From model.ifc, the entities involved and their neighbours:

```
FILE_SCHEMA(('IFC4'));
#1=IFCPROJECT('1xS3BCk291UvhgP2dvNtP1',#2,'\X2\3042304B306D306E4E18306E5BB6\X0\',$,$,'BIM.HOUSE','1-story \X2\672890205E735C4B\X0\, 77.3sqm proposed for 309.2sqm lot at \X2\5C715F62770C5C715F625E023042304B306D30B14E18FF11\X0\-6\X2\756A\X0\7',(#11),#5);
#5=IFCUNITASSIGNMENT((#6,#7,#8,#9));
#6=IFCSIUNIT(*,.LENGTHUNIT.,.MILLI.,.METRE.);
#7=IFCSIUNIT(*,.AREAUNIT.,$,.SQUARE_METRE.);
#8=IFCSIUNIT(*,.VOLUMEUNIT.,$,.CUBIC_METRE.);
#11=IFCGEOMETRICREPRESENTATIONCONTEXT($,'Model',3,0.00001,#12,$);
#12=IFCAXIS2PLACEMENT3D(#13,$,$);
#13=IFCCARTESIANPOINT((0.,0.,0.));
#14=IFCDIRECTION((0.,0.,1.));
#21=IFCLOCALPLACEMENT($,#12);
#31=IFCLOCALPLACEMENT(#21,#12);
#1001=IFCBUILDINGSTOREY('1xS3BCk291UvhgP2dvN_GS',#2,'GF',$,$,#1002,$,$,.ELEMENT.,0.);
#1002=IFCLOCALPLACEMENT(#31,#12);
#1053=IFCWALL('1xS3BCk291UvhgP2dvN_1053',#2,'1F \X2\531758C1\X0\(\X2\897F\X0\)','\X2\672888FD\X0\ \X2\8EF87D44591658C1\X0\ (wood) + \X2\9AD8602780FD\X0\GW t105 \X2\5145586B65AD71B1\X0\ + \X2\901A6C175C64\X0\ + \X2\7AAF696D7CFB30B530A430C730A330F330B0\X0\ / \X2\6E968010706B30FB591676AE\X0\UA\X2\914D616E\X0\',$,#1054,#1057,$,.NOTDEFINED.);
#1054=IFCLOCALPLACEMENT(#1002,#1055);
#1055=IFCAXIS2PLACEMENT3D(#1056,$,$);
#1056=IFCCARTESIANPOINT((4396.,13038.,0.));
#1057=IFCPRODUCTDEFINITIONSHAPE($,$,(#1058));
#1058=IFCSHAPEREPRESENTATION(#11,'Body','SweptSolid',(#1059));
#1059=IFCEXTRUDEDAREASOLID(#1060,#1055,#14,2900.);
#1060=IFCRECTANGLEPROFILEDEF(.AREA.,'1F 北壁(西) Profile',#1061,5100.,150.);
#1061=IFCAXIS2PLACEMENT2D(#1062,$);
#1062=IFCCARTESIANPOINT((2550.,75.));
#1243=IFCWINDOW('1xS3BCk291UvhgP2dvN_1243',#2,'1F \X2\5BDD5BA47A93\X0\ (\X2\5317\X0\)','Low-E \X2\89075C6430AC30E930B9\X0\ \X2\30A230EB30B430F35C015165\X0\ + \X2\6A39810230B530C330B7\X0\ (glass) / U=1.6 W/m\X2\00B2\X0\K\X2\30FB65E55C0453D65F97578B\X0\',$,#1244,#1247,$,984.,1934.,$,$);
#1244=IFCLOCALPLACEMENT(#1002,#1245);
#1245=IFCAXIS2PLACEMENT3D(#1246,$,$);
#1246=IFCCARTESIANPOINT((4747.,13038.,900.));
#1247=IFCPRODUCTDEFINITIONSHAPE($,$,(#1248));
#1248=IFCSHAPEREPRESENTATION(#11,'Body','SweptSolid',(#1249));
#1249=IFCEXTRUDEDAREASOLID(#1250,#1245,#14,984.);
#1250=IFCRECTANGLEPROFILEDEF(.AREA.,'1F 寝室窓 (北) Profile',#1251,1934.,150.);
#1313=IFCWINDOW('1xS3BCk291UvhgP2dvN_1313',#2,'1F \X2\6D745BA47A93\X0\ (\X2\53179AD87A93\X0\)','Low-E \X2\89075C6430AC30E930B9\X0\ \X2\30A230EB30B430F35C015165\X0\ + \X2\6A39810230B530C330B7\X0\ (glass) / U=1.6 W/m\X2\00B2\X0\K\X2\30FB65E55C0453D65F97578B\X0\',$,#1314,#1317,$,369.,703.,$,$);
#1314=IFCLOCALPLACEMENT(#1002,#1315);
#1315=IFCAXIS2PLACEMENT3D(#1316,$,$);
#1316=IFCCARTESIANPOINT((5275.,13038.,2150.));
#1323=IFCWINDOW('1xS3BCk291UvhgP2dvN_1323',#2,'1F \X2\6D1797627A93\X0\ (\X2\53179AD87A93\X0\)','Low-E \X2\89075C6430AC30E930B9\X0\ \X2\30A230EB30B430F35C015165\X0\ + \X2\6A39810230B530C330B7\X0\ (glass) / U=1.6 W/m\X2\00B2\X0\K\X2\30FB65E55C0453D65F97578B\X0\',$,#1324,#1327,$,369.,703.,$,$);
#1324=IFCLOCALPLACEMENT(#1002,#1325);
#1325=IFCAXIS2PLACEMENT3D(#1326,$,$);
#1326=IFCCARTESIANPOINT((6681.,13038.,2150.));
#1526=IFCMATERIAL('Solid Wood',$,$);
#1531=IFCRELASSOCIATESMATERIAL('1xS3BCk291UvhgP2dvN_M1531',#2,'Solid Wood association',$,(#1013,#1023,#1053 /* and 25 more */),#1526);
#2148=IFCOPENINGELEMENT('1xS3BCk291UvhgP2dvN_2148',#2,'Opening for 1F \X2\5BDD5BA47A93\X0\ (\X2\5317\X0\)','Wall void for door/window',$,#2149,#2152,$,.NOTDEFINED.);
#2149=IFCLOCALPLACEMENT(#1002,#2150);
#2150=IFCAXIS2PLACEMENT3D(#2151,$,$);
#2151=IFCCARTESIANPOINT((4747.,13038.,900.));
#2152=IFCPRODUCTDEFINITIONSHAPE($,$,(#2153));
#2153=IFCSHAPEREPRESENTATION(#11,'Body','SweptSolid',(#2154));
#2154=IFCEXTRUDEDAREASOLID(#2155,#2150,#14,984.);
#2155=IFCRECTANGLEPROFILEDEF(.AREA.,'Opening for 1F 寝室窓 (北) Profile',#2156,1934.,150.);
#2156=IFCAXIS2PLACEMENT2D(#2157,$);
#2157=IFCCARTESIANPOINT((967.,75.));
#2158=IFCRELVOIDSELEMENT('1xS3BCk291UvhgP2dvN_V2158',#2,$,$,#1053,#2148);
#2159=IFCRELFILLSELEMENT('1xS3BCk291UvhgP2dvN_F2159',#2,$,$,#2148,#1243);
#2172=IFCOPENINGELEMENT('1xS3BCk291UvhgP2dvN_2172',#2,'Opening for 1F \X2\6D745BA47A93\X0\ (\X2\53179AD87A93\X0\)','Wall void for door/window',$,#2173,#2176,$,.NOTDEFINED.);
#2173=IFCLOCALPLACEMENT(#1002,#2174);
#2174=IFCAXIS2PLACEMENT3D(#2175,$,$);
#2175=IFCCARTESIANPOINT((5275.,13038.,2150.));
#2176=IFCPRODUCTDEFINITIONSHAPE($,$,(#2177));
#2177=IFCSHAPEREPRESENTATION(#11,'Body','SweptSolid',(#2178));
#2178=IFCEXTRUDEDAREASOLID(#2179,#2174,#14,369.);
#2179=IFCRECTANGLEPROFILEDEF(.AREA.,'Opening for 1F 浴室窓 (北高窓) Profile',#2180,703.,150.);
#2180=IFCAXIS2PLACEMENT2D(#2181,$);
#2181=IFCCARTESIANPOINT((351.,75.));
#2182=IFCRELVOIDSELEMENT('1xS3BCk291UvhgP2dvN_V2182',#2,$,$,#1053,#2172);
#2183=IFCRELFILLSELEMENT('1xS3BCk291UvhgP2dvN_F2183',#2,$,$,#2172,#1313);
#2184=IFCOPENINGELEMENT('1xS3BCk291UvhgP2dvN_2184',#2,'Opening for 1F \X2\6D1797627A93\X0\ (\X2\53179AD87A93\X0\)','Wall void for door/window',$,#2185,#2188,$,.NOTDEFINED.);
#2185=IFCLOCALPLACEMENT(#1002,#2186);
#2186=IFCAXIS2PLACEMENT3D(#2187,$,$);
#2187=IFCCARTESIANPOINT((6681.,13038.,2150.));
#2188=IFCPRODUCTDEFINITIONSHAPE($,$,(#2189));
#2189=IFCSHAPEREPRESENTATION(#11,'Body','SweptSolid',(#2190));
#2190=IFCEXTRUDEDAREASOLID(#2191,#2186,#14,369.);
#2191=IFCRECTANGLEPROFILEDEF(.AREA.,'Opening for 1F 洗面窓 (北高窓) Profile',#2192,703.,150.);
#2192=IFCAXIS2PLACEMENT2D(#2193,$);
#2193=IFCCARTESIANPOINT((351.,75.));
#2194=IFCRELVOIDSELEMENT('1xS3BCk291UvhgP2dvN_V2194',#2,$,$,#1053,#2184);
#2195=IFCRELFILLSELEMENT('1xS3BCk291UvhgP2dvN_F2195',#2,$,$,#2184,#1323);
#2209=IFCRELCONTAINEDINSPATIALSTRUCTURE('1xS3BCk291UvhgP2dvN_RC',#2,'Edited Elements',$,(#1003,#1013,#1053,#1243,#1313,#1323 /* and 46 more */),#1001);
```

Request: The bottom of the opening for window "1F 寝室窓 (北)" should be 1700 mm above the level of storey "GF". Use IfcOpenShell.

```python
import numpy as np
import ifcopenshell
import ifcopenshell.api.geometry
import ifcopenshell.geom
import ifcopenshell.util.element
import ifcopenshell.util.placement
import ifcopenshell.util.shape
import ifcopenshell.util.unit

model = ifcopenshell.open("model.ifc")
unit_scale = ifcopenshell.util.unit.calculate_unit_scale(model)

window = model.by_guid("1xS3BCk291UvhgP2dvN_1243")
opening = window.FillsVoids[0].RelatingOpeningElement
storey = ifcopenshell.util.element.get_container(window, ifc_class="IfcBuildingStorey")
level = ifcopenshell.util.placement.get_local_placement(storey.ObjectPlacement)[2, 3]

# The opening's origin need not be at the sill, so measure its lowest point.
shape = ifcopenshell.geom.create_shape(ifcopenshell.geom.settings(), opening)
bottom = ifcopenshell.util.shape.get_shape_bottom_elevation(shape, shape.geometry) / unit_scale
dz = level + 1700.0 - bottom

shift = np.array([0.0, 0.0, dz])
# The window is not placed relative to its opening, so move both.
for product in (opening, window):
    matrix = ifcopenshell.util.placement.get_local_placement(product.ObjectPlacement)
    matrix[:3, 3] += shift
    ifcopenshell.api.geometry.edit_object_placement(model, product=product, matrix=matrix, is_si=False)

print(f"moved by {dz * unit_scale:+.3f} m")

model.write("model_v2.ifc")
```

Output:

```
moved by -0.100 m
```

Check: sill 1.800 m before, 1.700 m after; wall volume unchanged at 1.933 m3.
